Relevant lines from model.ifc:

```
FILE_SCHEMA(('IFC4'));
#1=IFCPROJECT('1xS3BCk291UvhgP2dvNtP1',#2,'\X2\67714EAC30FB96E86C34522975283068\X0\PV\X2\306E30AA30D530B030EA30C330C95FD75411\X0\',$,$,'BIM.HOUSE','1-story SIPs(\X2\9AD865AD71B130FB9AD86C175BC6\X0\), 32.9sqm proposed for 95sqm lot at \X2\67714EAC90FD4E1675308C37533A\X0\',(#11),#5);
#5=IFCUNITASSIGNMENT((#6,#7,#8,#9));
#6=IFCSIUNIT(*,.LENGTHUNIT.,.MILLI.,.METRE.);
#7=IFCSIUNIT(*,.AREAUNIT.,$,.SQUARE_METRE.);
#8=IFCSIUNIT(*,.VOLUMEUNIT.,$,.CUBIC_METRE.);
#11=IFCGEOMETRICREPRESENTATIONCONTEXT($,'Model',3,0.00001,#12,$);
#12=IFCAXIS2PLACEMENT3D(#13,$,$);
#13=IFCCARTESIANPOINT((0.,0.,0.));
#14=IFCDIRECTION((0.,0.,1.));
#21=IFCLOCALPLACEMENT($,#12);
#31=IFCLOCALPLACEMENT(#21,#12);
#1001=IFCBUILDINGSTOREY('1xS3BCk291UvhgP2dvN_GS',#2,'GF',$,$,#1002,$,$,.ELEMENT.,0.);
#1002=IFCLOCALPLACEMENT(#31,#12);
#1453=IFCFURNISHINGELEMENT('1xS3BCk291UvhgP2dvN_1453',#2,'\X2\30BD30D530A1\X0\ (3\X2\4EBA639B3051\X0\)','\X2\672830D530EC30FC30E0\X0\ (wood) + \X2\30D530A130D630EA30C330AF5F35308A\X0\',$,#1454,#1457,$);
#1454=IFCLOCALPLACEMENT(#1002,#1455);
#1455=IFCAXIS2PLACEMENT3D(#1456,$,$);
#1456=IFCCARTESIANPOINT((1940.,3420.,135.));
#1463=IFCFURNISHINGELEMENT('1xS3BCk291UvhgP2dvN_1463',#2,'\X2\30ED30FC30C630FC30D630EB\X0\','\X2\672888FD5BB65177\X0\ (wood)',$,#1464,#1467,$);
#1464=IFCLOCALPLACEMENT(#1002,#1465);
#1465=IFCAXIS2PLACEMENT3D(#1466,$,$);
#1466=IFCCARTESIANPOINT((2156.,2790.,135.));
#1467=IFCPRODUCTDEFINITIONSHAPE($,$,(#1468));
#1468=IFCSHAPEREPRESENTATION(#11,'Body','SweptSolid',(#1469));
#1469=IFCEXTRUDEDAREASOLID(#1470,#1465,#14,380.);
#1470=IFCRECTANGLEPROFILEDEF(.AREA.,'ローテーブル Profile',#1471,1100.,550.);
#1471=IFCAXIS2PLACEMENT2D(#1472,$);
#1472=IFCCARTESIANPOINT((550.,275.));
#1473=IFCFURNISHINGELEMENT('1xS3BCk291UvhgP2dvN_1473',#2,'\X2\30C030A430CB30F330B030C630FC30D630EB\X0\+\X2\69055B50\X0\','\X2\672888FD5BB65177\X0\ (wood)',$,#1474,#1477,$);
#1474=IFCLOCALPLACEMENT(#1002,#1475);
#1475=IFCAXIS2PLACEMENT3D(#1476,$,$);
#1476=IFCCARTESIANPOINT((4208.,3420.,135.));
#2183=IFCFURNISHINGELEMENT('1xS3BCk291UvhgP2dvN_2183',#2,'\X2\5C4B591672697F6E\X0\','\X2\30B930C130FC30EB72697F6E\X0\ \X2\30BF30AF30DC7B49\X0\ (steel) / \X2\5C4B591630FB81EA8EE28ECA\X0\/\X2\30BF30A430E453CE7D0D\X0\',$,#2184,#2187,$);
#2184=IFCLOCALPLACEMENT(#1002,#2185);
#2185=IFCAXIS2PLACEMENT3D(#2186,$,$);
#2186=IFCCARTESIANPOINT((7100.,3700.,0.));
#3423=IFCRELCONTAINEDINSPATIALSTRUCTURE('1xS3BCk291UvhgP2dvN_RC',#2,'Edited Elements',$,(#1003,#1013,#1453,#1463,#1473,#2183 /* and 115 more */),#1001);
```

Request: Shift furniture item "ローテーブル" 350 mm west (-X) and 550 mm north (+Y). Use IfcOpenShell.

```python
import ifcopenshell
import ifcopenshell.api.geometry
import ifcopenshell.util.placement

model = ifcopenshell.open("model.ifc")

item = model.by_id(1463)
matrix = ifcopenshell.util.placement.get_local_placement(item.ObjectPlacement)
matrix[0, 3] -= 350.0
matrix[1, 3] += 550.0
ifcopenshell.api.geometry.edit_object_placement(model, product=item, matrix=matrix, is_si=False)

print(ifcopenshell.util.placement.get_local_placement(item.ObjectPlacement).round(3) + 0.0)

model.write("model_v2.ifc")
```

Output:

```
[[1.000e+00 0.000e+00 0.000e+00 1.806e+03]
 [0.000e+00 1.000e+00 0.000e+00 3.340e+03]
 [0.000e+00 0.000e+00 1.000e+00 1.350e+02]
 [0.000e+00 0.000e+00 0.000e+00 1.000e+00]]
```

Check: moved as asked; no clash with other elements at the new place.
